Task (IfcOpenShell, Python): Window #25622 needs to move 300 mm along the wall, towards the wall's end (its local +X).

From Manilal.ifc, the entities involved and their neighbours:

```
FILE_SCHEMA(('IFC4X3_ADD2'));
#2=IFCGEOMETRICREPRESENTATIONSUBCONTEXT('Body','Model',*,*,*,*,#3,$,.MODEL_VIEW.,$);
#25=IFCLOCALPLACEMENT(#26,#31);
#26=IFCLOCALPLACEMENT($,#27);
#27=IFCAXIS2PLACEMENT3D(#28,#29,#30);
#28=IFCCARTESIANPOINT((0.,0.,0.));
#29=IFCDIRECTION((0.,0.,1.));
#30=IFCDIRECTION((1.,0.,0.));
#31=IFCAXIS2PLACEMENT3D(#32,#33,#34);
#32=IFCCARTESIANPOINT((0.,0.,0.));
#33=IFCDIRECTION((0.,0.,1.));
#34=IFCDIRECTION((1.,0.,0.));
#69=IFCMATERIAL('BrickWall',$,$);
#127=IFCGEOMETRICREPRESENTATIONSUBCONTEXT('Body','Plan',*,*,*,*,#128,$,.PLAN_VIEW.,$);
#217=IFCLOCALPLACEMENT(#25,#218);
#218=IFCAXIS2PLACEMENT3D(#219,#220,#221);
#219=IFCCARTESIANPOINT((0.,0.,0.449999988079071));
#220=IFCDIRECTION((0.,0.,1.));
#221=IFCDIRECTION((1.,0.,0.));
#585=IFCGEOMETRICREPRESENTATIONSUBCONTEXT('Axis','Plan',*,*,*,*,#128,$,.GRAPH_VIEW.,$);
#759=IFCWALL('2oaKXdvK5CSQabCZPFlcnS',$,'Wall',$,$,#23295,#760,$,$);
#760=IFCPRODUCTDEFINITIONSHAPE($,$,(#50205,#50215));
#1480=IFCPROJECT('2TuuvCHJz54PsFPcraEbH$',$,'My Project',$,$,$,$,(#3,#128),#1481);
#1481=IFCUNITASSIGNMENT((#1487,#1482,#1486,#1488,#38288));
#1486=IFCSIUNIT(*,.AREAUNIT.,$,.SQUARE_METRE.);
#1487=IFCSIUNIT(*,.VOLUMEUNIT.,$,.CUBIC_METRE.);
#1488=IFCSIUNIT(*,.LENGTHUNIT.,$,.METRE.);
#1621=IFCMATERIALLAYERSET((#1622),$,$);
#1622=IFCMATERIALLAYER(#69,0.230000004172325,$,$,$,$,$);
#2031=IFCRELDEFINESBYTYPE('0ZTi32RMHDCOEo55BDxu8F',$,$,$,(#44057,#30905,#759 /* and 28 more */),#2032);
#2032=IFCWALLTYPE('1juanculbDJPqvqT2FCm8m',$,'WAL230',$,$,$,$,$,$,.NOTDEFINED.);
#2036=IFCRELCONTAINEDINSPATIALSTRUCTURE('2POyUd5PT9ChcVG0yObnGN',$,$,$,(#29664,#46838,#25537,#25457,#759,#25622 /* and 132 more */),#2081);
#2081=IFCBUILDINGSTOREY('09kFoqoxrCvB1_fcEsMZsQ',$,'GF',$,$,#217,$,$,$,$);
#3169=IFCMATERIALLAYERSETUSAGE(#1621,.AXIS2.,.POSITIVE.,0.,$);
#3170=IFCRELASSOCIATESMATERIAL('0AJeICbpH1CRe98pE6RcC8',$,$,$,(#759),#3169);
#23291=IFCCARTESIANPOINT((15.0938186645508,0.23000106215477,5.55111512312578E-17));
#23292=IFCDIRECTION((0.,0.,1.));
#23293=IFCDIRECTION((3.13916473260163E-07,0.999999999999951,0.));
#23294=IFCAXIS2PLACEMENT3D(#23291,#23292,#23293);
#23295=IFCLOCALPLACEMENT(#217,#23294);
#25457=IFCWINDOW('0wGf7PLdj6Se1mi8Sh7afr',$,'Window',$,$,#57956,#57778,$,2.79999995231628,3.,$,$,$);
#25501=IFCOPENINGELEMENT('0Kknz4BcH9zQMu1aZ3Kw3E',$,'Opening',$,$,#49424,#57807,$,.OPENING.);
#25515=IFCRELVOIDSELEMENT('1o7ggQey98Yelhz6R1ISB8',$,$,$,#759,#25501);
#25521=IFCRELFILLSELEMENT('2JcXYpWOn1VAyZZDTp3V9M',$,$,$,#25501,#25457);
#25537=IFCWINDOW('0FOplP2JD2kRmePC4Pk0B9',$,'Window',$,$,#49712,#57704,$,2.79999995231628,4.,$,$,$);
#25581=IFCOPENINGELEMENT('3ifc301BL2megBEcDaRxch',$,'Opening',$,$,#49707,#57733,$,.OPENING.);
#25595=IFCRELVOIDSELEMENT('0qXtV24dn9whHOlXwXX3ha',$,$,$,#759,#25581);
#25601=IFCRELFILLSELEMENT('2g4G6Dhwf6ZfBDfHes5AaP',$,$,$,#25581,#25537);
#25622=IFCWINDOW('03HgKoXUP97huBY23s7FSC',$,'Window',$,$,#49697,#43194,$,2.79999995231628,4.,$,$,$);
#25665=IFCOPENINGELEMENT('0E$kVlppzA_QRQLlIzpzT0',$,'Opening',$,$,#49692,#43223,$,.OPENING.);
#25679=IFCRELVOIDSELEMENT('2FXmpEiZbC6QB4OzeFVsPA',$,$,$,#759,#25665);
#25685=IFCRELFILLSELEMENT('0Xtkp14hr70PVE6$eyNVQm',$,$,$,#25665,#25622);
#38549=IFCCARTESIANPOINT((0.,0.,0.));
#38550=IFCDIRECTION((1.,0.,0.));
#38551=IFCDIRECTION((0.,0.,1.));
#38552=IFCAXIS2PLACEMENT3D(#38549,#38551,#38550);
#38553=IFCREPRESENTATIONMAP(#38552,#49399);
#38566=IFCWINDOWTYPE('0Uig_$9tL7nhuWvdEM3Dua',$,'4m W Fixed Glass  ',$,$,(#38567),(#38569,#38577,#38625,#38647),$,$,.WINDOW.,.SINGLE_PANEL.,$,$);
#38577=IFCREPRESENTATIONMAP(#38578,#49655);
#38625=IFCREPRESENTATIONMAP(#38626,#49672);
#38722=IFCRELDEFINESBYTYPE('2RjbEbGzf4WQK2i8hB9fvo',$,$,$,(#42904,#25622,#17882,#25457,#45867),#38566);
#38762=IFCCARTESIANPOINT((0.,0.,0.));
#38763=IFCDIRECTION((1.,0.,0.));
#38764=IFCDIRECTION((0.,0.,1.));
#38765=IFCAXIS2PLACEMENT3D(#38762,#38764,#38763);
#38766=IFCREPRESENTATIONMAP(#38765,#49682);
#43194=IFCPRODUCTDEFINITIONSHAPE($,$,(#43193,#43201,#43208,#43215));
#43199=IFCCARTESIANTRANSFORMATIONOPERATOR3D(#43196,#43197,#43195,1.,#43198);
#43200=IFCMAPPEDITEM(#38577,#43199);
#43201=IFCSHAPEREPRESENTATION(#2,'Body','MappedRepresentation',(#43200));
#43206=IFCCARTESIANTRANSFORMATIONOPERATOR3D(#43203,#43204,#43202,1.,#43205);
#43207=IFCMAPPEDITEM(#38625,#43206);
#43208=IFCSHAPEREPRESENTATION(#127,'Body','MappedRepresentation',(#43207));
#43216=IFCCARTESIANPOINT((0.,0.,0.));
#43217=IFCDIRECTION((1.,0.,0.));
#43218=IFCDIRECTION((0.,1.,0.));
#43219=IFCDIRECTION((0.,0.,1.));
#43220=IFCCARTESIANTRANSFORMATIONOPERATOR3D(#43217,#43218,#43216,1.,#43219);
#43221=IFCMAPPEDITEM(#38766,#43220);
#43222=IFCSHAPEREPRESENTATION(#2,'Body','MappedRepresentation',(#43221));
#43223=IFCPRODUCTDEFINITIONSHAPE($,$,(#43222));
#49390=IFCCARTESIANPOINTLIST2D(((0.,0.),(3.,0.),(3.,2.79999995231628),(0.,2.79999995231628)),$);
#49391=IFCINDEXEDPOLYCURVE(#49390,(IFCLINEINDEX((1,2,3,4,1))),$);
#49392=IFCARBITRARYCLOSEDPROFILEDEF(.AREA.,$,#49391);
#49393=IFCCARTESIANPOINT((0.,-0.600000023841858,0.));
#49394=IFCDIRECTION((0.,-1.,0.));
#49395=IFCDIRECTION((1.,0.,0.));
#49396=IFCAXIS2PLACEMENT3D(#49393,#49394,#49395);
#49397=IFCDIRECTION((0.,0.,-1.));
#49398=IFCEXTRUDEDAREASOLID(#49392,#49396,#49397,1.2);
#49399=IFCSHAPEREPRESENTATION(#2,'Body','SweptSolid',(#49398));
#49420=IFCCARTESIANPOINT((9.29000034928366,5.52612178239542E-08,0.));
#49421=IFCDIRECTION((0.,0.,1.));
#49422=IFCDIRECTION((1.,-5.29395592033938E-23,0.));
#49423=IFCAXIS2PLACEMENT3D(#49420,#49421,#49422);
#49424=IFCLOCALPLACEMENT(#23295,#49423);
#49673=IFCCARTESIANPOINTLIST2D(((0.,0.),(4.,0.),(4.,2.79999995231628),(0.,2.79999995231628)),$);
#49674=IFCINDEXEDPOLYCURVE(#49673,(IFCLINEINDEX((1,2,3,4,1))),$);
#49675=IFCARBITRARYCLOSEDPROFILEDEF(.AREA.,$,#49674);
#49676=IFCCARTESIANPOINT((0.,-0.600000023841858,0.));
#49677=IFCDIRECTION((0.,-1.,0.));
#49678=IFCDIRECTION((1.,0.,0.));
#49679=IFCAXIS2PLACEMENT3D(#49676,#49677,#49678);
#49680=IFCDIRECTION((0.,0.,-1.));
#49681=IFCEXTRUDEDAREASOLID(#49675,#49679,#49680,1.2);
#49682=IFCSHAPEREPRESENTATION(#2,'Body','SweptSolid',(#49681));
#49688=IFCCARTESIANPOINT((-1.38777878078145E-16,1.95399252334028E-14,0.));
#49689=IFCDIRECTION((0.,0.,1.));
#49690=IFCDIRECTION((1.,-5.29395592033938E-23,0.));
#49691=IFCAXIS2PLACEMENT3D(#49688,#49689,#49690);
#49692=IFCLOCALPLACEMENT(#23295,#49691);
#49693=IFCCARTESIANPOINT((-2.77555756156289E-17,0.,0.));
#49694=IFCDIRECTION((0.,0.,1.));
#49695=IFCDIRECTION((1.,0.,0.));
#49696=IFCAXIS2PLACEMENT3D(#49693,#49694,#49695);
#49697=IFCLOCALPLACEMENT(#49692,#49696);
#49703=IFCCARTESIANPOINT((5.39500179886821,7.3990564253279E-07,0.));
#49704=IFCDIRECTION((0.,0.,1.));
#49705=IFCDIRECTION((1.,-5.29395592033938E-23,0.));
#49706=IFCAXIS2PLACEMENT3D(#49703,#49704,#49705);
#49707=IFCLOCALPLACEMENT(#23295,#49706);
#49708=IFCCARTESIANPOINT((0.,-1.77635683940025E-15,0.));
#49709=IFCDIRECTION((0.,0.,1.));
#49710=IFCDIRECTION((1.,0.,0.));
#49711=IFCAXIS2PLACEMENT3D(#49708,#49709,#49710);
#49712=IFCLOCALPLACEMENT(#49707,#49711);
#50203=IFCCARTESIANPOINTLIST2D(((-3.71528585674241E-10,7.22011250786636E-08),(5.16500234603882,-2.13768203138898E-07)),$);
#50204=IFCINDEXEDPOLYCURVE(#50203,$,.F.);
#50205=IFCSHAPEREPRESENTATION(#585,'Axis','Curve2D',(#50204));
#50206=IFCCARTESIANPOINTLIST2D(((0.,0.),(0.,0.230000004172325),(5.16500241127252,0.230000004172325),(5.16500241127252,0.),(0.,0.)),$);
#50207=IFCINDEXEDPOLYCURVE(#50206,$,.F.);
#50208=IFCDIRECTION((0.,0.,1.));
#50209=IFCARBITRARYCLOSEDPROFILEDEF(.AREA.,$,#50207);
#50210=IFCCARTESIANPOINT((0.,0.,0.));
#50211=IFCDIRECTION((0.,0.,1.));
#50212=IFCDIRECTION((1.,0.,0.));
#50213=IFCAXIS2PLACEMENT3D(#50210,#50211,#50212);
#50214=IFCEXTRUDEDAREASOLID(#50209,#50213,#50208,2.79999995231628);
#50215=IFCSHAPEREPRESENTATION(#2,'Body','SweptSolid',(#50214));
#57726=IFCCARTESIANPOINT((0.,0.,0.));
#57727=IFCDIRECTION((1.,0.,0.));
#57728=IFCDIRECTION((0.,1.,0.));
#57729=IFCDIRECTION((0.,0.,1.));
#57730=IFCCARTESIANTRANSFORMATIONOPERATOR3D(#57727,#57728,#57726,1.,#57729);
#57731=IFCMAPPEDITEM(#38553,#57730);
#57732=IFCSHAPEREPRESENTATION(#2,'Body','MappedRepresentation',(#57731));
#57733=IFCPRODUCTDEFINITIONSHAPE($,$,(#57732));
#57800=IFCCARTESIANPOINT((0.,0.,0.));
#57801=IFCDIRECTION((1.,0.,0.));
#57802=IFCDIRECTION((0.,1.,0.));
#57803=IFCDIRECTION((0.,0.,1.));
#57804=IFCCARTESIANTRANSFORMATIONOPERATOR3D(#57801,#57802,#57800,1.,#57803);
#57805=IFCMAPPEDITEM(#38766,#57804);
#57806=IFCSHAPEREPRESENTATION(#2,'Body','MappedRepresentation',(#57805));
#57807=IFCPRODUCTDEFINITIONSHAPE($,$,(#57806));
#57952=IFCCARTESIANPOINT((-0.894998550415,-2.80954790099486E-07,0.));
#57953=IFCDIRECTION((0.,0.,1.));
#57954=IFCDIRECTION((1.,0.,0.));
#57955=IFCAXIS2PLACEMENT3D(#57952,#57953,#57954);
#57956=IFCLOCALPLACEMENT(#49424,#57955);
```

```python
import ifcopenshell
import ifcopenshell.api.geometry
import ifcopenshell.util.placement

model = ifcopenshell.open("Manilal.ifc")

window = model.by_guid("03HgKoXUP97huBY23s7FSC")
opening = window.FillsVoids[0].RelatingOpeningElement
wall = opening.VoidsElements[0].RelatingBuildingElement

wall_matrix = ifcopenshell.util.placement.get_local_placement(wall.ObjectPlacement)
shift = wall_matrix[:3, 0] * 0.3
before = ifcopenshell.util.placement.get_local_placement(window.ObjectPlacement)[:3, 3].copy()

# The window is placed relative to its opening, so it follows when the opening moves.
matrix = ifcopenshell.util.placement.get_local_placement(opening.ObjectPlacement)
matrix[:3, 3] += shift
ifcopenshell.api.geometry.edit_object_placement(
    model, product=opening, matrix=matrix, is_si=False, should_transform_children=True
)

after = ifcopenshell.util.placement.get_local_placement(window.ObjectPlacement)[:3, 3]
print("window moved by", (after - before).round(3) + 0.0)

model.write("Manilal_rev.ifc")
```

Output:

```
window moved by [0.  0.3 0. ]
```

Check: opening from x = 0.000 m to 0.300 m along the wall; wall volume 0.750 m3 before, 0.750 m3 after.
